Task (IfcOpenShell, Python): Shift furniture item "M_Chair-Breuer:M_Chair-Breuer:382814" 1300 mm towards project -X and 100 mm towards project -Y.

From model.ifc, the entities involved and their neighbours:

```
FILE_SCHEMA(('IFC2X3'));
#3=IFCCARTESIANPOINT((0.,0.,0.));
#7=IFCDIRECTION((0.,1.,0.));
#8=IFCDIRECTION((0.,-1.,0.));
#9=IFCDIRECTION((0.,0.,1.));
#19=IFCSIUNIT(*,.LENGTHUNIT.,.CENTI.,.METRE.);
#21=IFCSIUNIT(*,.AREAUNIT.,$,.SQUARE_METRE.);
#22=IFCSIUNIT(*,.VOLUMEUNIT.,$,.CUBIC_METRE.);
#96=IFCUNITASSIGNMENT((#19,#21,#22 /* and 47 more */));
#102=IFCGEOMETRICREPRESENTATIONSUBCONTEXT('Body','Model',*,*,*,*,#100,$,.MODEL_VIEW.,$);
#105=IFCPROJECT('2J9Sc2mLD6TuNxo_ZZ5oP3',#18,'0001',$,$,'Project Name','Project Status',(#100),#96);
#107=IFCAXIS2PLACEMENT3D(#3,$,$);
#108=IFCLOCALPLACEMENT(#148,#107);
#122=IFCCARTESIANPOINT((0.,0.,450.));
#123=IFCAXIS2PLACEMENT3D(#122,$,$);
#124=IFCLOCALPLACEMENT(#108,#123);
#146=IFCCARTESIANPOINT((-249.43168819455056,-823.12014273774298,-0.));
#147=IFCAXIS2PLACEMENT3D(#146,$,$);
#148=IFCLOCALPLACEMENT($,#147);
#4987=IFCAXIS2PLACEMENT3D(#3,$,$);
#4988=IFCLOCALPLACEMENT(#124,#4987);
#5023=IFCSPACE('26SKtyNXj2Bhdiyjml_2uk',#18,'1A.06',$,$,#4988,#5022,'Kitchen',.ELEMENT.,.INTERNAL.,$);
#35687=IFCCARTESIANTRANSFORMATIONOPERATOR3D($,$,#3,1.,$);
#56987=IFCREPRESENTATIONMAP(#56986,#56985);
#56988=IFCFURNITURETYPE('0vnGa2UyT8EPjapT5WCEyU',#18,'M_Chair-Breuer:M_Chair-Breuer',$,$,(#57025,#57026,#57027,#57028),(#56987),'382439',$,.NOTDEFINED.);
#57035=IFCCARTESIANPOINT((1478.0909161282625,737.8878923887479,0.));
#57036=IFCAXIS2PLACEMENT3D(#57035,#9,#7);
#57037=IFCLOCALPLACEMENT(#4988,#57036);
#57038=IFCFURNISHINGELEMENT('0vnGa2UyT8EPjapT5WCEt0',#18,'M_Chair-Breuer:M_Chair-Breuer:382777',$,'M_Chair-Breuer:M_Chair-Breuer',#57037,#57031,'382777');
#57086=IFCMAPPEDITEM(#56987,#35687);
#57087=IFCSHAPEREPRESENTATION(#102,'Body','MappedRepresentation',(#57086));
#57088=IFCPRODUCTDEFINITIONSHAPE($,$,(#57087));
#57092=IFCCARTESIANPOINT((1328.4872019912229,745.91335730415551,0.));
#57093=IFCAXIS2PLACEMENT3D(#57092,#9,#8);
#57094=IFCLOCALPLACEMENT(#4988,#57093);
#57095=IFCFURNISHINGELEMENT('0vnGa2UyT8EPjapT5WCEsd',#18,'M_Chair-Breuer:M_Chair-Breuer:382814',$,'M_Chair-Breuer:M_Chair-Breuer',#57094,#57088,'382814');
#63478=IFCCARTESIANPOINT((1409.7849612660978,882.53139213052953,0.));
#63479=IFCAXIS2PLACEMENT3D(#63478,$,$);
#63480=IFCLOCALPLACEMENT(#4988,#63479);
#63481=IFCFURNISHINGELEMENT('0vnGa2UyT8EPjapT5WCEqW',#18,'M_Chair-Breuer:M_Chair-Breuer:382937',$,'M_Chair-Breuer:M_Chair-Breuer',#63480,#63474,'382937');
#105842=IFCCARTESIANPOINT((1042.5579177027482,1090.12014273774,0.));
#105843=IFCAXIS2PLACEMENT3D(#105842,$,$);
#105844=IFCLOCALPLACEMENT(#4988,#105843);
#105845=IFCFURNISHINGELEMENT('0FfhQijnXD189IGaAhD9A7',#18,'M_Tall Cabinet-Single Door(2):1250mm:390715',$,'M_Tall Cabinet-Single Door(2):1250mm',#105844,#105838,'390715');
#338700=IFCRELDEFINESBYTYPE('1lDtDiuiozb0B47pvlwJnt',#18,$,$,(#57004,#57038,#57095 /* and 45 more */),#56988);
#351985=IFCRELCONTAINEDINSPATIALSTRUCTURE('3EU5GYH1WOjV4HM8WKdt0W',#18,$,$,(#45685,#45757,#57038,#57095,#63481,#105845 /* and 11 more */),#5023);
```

```python
import ifcopenshell
import ifcopenshell.api.geometry
import ifcopenshell.util.placement
import ifcopenshell.util.unit

model = ifcopenshell.open("model.ifc")
unit_scale = ifcopenshell.util.unit.calculate_unit_scale(model)

item = model.by_guid("0vnGa2UyT8EPjapT5WCEsd")
matrix = ifcopenshell.util.placement.get_local_placement(item.ObjectPlacement)
matrix[0, 3] -= 1.3 / unit_scale
matrix[1, 3] -= 0.1 / unit_scale
ifcopenshell.api.geometry.edit_object_placement(model, product=item, matrix=matrix, is_si=False)

print(ifcopenshell.util.placement.get_local_placement(item.ObjectPlacement).round(3) + 0.0)

model.write("model_rev.ifc")
```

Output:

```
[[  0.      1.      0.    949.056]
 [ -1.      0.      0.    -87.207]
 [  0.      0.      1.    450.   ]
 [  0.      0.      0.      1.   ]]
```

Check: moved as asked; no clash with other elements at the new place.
